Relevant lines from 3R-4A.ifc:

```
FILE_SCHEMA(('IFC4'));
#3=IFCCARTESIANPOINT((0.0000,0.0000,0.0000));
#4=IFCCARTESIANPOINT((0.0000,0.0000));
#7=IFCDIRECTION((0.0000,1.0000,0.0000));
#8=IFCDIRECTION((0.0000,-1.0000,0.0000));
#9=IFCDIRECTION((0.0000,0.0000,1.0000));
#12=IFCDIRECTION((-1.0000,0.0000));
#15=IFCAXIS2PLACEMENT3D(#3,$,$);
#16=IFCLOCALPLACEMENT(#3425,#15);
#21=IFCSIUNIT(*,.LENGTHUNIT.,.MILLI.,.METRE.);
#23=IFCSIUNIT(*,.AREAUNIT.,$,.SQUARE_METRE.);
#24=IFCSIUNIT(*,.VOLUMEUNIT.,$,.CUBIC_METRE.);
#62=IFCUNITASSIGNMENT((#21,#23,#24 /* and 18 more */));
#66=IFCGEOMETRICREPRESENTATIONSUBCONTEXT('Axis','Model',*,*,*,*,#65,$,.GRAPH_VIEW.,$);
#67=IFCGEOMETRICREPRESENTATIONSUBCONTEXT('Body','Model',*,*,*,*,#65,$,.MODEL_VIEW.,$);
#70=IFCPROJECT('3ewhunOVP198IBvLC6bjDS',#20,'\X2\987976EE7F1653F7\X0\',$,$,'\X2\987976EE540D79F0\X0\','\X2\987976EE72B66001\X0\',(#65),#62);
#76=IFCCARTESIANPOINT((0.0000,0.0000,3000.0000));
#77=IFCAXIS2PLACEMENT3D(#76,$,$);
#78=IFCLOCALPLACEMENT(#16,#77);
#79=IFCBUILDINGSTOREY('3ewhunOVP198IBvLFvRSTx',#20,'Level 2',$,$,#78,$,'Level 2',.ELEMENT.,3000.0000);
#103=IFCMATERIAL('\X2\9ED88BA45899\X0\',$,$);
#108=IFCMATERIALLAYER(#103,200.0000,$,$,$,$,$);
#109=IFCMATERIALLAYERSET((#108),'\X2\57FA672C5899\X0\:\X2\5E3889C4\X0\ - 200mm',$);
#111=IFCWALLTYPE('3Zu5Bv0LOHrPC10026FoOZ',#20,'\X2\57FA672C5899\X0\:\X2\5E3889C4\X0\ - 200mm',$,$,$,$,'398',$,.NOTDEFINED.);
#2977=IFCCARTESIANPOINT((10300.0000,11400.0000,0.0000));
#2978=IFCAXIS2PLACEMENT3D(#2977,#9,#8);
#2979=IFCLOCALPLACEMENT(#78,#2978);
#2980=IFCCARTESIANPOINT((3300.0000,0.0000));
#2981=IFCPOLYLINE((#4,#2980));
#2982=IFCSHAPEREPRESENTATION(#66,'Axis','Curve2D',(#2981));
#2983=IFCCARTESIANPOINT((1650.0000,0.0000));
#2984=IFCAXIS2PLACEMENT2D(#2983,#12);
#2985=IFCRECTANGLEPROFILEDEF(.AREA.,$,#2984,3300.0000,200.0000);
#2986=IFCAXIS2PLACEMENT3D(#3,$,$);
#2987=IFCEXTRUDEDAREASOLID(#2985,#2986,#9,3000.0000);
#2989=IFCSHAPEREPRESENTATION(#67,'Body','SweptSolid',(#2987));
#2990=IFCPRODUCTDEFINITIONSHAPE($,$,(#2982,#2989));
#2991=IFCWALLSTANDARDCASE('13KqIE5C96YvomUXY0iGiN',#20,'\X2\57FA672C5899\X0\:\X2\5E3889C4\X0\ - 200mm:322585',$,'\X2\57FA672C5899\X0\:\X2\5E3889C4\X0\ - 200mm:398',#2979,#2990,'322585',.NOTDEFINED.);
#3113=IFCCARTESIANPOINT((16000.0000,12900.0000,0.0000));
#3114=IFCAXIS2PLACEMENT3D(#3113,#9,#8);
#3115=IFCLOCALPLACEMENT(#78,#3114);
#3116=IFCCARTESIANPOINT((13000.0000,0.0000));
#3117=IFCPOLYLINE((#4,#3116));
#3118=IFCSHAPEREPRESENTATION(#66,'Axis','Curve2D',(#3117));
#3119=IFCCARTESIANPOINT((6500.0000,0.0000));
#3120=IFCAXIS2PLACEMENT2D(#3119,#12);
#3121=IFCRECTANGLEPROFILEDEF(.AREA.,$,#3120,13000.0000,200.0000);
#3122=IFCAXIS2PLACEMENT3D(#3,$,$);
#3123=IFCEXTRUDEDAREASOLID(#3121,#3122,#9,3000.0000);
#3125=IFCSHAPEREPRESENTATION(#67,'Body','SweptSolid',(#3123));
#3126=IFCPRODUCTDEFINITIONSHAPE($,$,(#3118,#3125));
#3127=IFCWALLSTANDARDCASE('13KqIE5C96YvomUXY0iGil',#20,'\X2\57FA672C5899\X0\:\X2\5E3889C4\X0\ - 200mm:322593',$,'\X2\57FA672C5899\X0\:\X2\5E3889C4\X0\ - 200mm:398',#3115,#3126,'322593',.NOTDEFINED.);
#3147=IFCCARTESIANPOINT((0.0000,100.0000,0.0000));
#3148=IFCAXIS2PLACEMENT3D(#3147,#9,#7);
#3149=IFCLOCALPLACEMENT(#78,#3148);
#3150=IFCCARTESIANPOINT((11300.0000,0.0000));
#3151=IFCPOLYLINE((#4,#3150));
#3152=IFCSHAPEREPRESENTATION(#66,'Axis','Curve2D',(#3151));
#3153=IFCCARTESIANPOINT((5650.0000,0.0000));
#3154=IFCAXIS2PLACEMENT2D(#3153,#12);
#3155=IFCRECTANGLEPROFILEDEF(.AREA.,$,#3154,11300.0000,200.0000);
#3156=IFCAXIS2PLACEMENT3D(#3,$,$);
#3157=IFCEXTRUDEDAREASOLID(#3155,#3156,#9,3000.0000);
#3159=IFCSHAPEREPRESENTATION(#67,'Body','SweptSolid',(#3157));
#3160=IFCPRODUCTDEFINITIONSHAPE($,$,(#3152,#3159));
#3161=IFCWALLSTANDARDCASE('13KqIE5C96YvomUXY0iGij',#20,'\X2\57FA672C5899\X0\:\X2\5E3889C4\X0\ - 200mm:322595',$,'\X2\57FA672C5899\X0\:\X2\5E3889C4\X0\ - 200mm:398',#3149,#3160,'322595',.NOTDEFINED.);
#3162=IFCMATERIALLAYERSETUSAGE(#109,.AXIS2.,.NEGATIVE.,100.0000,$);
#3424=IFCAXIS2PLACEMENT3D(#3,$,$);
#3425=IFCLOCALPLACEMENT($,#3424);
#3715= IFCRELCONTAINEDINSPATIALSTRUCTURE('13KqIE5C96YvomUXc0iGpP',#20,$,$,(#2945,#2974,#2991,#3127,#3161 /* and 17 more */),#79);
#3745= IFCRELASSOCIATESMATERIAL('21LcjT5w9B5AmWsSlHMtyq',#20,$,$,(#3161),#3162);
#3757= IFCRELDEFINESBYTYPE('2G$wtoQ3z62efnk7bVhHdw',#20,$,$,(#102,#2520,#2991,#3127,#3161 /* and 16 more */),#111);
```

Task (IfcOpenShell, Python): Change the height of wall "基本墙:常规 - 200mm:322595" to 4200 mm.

```python
import ifcopenshell
import ifcopenshell.geom
import ifcopenshell.util.representation
import ifcopenshell.util.shape

model = ifcopenshell.open("3R-4A.ifc")
settings = ifcopenshell.geom.settings()


def volume(element):
    """Net volume in cubic metres, openings subtracted."""
    shape = ifcopenshell.geom.create_shape(settings, element)
    return ifcopenshell.util.shape.get_volume(shape.geometry)


wall = model.by_id(3161)
before = volume(wall)

body = ifcopenshell.util.representation.get_representation(wall, "Model", "Body")
solid = body.Items[0]
old_height = solid.Depth
solid.Depth = 4200.0
after = volume(wall)

print(f"height {old_height:g} -> {solid.Depth:g}, volume {before:.3f} -> {after:.3f} m3")

model.write("3R-4A_v2.ifc")
```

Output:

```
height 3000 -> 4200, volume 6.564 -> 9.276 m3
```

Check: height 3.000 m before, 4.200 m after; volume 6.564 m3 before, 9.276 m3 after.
